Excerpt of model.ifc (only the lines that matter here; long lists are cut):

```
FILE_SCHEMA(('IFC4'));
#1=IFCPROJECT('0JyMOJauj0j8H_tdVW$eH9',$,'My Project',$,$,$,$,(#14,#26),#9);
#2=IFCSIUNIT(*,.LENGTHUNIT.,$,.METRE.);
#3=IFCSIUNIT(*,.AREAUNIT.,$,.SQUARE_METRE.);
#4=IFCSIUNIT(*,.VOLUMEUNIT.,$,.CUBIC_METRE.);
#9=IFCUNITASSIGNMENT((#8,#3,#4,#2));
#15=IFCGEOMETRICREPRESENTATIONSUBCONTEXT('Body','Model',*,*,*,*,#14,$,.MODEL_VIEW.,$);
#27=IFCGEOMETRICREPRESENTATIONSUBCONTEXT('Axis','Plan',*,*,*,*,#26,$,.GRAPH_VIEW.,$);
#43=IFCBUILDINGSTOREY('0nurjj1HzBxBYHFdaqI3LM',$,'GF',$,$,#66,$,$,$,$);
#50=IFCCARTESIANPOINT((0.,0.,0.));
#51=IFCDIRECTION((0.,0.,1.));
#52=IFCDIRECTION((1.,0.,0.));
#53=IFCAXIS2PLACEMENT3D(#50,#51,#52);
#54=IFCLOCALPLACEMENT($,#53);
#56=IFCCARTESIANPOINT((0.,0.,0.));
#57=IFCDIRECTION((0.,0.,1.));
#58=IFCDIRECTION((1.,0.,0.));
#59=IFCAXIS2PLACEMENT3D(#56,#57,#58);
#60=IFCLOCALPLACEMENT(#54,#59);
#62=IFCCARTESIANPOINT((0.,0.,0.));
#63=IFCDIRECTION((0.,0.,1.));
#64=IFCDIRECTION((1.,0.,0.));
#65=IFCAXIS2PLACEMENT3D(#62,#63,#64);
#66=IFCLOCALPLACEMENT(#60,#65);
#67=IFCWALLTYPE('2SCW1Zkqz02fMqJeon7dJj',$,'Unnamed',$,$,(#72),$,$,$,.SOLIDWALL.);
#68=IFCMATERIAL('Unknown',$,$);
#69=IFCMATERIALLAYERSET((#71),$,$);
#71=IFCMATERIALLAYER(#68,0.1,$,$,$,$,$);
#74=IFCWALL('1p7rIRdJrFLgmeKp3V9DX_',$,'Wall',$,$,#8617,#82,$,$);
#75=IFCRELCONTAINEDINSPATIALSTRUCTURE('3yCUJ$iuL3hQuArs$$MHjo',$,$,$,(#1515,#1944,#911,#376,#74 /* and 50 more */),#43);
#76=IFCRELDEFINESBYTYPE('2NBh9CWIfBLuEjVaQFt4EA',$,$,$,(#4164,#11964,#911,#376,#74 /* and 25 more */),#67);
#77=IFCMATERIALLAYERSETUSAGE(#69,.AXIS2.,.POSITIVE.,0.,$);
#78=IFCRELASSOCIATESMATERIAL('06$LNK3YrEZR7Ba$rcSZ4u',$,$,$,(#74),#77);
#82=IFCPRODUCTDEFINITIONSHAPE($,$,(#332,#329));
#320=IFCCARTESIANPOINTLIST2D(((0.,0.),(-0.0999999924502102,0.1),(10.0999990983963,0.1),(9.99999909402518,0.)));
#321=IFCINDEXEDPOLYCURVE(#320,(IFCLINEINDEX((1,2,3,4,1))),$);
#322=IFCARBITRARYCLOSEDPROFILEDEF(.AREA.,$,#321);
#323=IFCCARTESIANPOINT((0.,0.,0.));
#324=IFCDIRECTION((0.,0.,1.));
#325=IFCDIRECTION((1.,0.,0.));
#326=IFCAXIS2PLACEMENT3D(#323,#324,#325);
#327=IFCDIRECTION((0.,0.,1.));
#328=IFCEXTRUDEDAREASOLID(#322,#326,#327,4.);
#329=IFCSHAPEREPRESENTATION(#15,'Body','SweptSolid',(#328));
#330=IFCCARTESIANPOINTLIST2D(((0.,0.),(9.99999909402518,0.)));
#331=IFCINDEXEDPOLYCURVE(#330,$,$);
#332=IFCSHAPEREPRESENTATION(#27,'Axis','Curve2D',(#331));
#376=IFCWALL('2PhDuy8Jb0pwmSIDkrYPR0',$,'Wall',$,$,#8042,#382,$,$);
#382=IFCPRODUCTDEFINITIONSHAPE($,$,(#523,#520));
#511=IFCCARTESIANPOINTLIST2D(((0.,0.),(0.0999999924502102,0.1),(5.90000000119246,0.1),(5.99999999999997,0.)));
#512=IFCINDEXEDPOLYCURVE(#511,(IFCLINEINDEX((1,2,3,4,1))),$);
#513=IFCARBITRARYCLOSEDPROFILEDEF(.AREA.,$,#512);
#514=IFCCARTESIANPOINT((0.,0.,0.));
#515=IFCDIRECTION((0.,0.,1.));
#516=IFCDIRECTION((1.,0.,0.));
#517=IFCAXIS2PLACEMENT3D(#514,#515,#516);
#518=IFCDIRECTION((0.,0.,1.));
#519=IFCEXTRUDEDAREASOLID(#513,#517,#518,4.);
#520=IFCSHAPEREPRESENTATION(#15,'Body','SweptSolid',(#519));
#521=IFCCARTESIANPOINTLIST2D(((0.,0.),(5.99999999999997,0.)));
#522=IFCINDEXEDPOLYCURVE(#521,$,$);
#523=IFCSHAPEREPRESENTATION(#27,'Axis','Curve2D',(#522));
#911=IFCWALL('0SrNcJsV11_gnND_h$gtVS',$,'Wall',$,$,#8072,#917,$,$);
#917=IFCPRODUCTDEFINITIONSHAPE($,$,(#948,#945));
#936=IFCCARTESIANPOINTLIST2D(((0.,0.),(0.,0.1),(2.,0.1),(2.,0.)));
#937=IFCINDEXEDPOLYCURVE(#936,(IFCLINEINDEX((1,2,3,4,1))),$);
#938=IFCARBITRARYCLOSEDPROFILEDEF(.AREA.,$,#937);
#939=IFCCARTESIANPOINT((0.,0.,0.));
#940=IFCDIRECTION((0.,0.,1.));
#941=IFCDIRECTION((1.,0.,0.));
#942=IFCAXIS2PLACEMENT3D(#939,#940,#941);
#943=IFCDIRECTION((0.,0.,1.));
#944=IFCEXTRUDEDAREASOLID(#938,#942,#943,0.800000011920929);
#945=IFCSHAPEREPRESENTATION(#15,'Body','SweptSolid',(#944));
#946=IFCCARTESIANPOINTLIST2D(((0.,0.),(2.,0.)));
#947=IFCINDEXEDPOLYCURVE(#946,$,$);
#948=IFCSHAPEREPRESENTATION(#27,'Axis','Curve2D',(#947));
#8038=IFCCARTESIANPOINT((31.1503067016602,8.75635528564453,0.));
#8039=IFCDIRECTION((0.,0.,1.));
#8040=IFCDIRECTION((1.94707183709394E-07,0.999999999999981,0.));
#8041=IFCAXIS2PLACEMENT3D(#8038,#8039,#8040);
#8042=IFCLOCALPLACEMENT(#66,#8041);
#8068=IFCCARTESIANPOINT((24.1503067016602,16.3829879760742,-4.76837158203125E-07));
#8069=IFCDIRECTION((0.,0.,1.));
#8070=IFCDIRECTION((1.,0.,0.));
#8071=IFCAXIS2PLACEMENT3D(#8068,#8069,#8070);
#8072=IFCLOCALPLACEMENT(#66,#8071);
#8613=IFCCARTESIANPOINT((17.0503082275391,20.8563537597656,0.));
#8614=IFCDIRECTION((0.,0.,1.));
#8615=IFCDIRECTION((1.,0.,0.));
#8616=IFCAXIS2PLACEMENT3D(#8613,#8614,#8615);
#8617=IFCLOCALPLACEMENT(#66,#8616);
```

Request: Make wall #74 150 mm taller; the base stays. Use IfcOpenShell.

```python
import ifcopenshell
import ifcopenshell.geom
import ifcopenshell.util.representation
import ifcopenshell.util.shape
import ifcopenshell.util.unit

model = ifcopenshell.open("model.ifc")
unit_scale = ifcopenshell.util.unit.calculate_unit_scale(model)
settings = ifcopenshell.geom.settings()


def volume(element):
    """Net volume in cubic metres, openings subtracted."""
    shape = ifcopenshell.geom.create_shape(settings, element)
    return ifcopenshell.util.shape.get_volume(shape.geometry)


wall = model.by_guid("1p7rIRdJrFLgmeKp3V9DX_")
before = volume(wall)

body = ifcopenshell.util.representation.get_representation(wall, "Model", "Body")
solid = body.Items[0]
old_height = solid.Depth
solid.Depth += 0.15 / unit_scale
after = volume(wall)

print(f"height {old_height:g} -> {solid.Depth:g}, volume {before:.3f} -> {after:.3f} m3")

model.write("model_rev.ifc")
```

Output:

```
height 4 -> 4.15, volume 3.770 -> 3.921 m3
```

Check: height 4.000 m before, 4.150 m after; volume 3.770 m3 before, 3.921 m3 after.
